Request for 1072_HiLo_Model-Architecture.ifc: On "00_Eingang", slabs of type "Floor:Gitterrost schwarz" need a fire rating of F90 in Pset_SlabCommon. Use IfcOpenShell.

First a look at what the model holds.

```python
import ifcopenshell
import ifcopenshell.util.element

model = ifcopenshell.open("1072_HiLo_Model-Architecture.ifc")
print(model.schema)
storey = next(s for s in model.by_type("IfcBuildingStorey") if s.Name == "00_Eingang")
slabs = [e for e in ifcopenshell.util.element.get_decomposition(storey) if e.is_a("IfcSlab")]
seen = {}
for e in slabs:
    element_type = ifcopenshell.util.element.get_type(e)
    key = (element_type.Name if element_type != e and element_type else None, ifcopenshell.util.element.get_pset(e, "Pset_SlabCommon", "FireRating"))
    seen[key] = seen.get(key, 0) + 1
for (name, value), count in sorted(seen.items(), key=str):
    print(count, "x", name, "|", value)
```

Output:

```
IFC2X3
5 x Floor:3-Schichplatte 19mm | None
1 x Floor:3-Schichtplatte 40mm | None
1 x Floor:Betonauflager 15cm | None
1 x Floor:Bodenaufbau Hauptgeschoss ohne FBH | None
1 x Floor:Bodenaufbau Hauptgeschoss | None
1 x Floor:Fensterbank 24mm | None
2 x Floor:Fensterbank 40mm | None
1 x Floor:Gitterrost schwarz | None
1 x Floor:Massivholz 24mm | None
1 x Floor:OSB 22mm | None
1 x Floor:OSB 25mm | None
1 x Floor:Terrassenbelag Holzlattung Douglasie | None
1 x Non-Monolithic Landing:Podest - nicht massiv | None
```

```python
import ifcopenshell
import ifcopenshell.api.pset
import ifcopenshell.util.element

model = ifcopenshell.open("1072_HiLo_Model-Architecture.ifc")

storey = next(s for s in model.by_type("IfcBuildingStorey") if s.Name == "00_Eingang")
slabs = [e for e in ifcopenshell.util.element.get_decomposition(storey) if e.is_a("IfcSlab")]

count = 0
for e in slabs:
    element_type = ifcopenshell.util.element.get_type(e)
    if element_type in (None, e) or element_type.Name != "Floor:Gitterrost schwarz":
        continue
    # add_pset returns the element's existing set when there is one.
    pset = ifcopenshell.api.pset.add_pset(model, product=e, name="Pset_SlabCommon")
    ifcopenshell.api.pset.edit_pset(model, pset=pset, properties={"FireRating": "F90"})
    count += 1

print(count, "slabs updated")

model.write("1072_HiLo_Model-Architecture_v2.ifc")
```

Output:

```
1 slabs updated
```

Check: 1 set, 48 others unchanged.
